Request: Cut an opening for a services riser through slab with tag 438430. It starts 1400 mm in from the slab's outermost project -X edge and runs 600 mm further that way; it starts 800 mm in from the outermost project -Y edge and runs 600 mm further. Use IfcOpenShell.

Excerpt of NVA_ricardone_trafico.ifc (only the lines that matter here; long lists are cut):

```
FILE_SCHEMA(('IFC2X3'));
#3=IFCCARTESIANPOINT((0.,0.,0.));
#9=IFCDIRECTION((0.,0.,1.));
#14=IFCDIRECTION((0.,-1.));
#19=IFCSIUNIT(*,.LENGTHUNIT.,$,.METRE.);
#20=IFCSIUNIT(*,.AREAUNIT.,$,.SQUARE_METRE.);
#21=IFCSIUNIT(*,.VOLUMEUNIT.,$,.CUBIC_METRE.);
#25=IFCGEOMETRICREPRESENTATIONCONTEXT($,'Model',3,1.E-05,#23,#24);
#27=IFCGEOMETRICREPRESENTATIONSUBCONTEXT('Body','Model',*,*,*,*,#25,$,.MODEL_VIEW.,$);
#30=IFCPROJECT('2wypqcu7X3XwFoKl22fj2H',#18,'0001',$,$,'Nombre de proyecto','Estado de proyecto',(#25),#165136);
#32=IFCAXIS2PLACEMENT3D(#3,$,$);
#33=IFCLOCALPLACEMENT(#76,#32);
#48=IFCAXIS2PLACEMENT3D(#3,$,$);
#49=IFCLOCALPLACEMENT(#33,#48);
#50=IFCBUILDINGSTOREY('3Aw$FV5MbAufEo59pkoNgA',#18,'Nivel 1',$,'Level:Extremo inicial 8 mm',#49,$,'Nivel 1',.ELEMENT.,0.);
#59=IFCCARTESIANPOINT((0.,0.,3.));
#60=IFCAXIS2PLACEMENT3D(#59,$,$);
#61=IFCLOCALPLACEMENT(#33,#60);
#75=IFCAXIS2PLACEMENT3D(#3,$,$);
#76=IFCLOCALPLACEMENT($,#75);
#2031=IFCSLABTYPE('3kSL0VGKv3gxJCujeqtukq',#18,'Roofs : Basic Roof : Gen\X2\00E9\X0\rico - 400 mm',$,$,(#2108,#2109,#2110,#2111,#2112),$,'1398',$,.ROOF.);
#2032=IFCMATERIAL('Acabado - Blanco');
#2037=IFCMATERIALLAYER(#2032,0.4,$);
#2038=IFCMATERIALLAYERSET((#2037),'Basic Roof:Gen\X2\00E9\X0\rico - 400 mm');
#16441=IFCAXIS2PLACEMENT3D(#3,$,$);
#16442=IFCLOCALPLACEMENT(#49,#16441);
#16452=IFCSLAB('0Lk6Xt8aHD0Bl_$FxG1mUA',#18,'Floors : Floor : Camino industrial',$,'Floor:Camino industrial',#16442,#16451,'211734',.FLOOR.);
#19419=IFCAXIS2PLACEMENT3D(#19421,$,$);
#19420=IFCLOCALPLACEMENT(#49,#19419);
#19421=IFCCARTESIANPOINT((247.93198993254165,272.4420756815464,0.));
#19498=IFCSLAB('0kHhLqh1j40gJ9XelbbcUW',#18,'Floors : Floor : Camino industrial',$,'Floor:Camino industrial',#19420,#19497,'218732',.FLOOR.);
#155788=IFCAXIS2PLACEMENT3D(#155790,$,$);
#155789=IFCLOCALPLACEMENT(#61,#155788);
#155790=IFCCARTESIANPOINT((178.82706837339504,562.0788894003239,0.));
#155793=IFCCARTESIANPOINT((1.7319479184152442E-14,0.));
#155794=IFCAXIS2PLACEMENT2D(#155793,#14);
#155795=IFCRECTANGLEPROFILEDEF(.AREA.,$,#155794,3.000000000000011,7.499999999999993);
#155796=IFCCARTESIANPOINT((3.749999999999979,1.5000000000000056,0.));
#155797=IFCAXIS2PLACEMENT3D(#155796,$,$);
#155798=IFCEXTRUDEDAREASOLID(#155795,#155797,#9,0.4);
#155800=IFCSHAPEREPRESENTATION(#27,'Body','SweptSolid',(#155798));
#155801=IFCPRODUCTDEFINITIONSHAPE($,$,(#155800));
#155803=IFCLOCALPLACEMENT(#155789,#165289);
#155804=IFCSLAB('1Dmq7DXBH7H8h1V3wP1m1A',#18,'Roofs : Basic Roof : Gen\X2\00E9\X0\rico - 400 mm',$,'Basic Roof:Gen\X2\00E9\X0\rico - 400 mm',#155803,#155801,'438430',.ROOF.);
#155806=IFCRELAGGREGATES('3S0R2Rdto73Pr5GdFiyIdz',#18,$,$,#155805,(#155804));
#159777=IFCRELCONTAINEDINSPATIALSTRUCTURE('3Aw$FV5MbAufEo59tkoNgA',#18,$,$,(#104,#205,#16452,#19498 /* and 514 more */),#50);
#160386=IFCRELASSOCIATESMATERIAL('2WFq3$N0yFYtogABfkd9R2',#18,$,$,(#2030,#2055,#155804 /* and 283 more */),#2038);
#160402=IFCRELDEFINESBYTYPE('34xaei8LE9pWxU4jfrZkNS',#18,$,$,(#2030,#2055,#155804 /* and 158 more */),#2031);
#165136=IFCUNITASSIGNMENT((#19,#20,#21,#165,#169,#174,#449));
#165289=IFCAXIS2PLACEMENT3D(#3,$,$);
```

```python
import numpy as np
import ifcopenshell
import ifcopenshell.api.feature
import ifcopenshell.api.geometry
import ifcopenshell.api.root
import ifcopenshell.geom
import ifcopenshell.util.placement
import ifcopenshell.util.representation
import ifcopenshell.util.shape
import ifcopenshell.util.unit

model = ifcopenshell.open("NVA_ricardone_trafico.ifc")
unit_scale = ifcopenshell.util.unit.calculate_unit_scale(model)
settings = ifcopenshell.geom.settings()


def volume(element):
    """Net volume in cubic metres, openings subtracted."""
    shape = ifcopenshell.geom.create_shape(settings, element)
    return ifcopenshell.util.shape.get_volume(shape.geometry)


slab = model.by_guid("1Dmq7DXBH7H8h1V3wP1m1A")
before = volume(slab)

# Extent in the slab's own axes, in metres. The edges named are its -X and -Y sides.
slab_shape = ifcopenshell.geom.create_shape(settings, slab)
vertices = ifcopenshell.util.shape.get_vertices(slab_shape.geometry)
x_min, y_min, bottom = vertices.min(axis=0)
top = vertices[:, 2].max()

opening = ifcopenshell.api.root.create_entity(model, ifc_class="IfcOpeningElement", name="Services riser opening")
context = ifcopenshell.util.representation.get_context(model, "Model", "Body", "MODEL_VIEW")
width, depth = 0.6, 0.6
outline = [(0.0, 0.0), (width, 0.0), (width, depth), (0.0, depth), (0.0, 0.0)]
# Overshoot both faces by 50 mm so the cut is clean.
shape = ifcopenshell.api.geometry.add_slab_representation(
    model, context=context, depth=top - bottom + 0.1, polyline=outline
)
ifcopenshell.api.geometry.assign_representation(model, product=opening, representation=shape)

matrix = ifcopenshell.util.placement.get_local_placement(slab.ObjectPlacement)
matrix[:, 3] = matrix @ np.append(np.array([x_min + 1.4, y_min + 0.8, bottom - 0.05]) / unit_scale, 1.0)
ifcopenshell.api.geometry.edit_object_placement(model, product=opening, matrix=matrix, is_si=False)
ifcopenshell.api.feature.add_feature(model, feature=opening, element=slab)

after = volume(slab)

print(f"slab volume {before:.3f} -> {after:.3f} m3")

model.write("NVA_ricardone_trafico_v2.ifc")
```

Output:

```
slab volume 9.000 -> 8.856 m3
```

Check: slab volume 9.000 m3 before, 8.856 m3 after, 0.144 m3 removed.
